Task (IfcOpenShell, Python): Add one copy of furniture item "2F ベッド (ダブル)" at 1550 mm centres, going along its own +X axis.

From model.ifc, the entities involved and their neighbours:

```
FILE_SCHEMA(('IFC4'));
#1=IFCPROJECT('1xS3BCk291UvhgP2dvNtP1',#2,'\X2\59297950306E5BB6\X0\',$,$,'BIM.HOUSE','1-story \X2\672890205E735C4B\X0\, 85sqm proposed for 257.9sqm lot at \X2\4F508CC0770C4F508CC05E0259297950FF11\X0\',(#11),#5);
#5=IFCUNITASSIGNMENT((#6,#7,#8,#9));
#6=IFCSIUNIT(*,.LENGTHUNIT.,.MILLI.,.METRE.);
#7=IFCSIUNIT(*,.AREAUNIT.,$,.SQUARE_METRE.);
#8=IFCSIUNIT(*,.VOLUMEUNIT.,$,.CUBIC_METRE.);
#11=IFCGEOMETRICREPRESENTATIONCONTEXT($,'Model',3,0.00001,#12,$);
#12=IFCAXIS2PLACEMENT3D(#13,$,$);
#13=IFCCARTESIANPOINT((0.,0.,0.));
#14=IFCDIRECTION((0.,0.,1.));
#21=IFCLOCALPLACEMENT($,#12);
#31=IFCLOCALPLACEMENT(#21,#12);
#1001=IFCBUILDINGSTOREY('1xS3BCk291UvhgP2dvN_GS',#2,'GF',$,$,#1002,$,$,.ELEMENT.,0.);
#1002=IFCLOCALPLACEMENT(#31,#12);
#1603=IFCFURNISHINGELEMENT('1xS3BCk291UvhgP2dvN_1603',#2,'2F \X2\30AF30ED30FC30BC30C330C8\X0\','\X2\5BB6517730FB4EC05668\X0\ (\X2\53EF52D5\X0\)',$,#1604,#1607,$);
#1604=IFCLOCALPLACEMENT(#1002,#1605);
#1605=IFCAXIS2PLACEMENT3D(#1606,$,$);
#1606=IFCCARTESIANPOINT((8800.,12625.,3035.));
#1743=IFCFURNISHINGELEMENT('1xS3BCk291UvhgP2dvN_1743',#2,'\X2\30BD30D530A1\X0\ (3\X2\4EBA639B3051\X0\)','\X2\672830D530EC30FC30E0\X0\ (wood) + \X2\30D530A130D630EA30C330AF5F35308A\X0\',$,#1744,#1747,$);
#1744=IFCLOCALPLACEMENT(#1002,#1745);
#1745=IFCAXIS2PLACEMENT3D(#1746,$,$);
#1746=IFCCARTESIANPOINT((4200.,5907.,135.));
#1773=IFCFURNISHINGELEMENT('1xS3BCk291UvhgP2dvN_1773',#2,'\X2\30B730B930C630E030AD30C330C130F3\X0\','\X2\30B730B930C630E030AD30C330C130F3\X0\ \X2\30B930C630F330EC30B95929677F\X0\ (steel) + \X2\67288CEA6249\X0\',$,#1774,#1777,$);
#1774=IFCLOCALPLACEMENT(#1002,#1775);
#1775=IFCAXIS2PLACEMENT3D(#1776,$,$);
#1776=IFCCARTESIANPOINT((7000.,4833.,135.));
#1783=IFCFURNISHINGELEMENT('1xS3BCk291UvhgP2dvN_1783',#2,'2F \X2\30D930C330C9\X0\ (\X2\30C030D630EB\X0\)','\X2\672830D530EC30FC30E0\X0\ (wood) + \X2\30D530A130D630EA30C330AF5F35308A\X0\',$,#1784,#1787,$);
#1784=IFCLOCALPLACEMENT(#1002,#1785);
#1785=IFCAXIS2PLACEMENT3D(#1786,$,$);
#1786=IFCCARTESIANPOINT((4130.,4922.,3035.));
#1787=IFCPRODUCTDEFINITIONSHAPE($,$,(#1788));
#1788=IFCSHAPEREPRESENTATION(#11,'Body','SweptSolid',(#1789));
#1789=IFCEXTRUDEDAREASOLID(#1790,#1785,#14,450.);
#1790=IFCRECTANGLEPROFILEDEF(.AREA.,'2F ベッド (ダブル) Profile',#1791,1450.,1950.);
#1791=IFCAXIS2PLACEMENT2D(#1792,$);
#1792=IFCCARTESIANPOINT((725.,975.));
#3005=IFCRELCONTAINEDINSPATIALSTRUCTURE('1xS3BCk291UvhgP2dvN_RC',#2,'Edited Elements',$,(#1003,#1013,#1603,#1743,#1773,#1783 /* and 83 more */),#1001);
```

```python
import ifcopenshell
import ifcopenshell.api.geometry
import ifcopenshell.api.root
import ifcopenshell.util.element
import ifcopenshell.util.placement
import ifcopenshell.util.unit

model = ifcopenshell.open("model.ifc")
unit_scale = ifcopenshell.util.unit.calculate_unit_scale(model)


def reuse_history(source, copy):
    """copy_class also copies each property set's owner history, people and application; keep the originals."""
    for rel in copy.IsDefinedBy:
        if rel.is_a("IfcRelDefinesByProperties") and (history := rel.RelatingPropertyDefinition.OwnerHistory):
            rel.RelatingPropertyDefinition.OwnerHistory = source.OwnerHistory
            ifcopenshell.util.element.remove_deep2(model, history)


source = model.by_guid("1xS3BCk291UvhgP2dvN_1783")
base = ifcopenshell.util.placement.get_local_placement(source.ObjectPlacement)
step = base[:3, 0] * 1.55 / unit_scale

for i in range(1, 2):
    copy = ifcopenshell.api.root.copy_class(model, product=source)
    copy.Representation = ifcopenshell.util.element.copy_deep(
        model, source.Representation, exclude=["IfcGeometricRepresentationContext", "IfcRepresentationMap"]
    )
    reuse_history(source, copy)
    matrix = base.copy()
    matrix[:3, 3] += i * step
    print("added at", matrix[:3, 3].round(3) + 0.0)
    ifcopenshell.api.geometry.edit_object_placement(model, product=copy, matrix=matrix, is_si=False)

model.write("model_edited.ifc")
```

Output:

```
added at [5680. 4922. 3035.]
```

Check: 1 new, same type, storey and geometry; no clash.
